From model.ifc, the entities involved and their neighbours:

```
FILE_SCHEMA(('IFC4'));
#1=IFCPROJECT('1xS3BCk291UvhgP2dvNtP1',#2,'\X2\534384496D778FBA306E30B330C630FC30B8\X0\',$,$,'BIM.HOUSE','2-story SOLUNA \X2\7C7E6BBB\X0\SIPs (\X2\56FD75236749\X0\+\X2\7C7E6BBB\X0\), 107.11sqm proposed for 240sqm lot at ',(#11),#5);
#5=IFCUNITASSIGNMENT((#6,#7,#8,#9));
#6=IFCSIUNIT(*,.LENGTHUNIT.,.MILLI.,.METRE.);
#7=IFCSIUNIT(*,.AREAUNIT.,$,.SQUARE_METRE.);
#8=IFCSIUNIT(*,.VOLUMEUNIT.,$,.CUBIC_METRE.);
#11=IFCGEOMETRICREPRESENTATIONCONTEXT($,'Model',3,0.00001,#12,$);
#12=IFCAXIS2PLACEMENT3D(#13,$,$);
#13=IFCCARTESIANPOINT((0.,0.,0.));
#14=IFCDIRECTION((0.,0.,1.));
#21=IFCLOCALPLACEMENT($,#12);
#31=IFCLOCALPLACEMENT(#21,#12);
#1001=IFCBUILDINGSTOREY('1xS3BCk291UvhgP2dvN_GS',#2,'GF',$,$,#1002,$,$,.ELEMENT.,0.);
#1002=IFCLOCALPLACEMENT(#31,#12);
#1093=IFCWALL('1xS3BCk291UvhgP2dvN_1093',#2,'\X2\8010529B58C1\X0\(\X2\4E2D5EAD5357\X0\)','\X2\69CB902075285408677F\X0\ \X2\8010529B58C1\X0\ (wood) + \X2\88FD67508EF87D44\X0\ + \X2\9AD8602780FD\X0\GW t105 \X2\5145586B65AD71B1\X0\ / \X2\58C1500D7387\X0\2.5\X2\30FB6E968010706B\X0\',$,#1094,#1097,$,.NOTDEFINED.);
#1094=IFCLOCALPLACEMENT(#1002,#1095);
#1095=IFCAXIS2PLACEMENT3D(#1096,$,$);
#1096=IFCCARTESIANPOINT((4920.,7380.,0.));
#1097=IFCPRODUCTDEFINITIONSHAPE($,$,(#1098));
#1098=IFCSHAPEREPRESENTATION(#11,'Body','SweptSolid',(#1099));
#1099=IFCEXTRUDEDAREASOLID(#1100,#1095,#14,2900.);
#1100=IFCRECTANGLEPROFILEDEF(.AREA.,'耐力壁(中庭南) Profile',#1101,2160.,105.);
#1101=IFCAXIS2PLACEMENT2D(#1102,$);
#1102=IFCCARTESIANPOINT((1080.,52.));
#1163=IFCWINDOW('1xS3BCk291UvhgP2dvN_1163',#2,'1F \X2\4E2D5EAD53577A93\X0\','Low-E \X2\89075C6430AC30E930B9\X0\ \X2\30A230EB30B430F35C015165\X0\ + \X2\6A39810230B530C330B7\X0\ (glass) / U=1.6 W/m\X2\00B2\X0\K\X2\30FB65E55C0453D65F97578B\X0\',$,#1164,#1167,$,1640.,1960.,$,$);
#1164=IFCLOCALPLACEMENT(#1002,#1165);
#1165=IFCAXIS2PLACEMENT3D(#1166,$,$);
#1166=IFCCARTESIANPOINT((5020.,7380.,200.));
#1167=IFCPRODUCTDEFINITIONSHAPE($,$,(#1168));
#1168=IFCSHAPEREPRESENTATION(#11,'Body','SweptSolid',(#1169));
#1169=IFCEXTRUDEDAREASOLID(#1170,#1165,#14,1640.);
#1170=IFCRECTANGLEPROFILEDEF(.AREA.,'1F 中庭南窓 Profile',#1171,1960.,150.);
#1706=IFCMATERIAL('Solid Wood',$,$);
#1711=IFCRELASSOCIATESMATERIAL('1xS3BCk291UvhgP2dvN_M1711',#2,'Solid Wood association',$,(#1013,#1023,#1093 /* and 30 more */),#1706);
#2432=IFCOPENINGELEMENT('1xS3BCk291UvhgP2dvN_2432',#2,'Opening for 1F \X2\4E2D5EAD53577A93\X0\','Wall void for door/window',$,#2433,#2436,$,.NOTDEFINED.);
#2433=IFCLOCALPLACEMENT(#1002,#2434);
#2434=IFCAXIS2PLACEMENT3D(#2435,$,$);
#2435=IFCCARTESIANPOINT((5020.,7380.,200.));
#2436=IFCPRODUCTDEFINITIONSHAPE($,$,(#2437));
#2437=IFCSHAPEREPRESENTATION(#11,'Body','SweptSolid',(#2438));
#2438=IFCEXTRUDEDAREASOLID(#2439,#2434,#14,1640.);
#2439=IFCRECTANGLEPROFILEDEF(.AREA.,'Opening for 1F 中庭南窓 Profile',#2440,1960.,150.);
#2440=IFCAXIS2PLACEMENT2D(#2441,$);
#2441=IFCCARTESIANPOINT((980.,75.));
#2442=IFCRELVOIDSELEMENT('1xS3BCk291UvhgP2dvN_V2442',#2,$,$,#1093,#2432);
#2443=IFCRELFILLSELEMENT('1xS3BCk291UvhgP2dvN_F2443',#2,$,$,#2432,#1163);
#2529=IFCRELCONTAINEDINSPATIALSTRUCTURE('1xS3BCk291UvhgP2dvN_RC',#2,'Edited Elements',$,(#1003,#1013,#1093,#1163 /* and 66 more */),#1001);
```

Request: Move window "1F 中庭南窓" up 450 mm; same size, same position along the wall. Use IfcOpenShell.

```python
import numpy as np
import ifcopenshell
import ifcopenshell.api.geometry
import ifcopenshell.util.placement
import ifcopenshell.util.unit

model = ifcopenshell.open("model.ifc")
unit_scale = ifcopenshell.util.unit.calculate_unit_scale(model)

window = model.by_guid("1xS3BCk291UvhgP2dvN_1163")
opening = window.FillsVoids[0].RelatingOpeningElement
dz = 450.0

shift = np.array([0.0, 0.0, dz])
# The window is not placed relative to its opening, so move both.
for product in (opening, window):
    matrix = ifcopenshell.util.placement.get_local_placement(product.ObjectPlacement)
    matrix[:3, 3] += shift
    ifcopenshell.api.geometry.edit_object_placement(model, product=product, matrix=matrix, is_si=False)

print(f"moved by {dz * unit_scale:+.3f} m")

model.write("model_v2.ifc")
```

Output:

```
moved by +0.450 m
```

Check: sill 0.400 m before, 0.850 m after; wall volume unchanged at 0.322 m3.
